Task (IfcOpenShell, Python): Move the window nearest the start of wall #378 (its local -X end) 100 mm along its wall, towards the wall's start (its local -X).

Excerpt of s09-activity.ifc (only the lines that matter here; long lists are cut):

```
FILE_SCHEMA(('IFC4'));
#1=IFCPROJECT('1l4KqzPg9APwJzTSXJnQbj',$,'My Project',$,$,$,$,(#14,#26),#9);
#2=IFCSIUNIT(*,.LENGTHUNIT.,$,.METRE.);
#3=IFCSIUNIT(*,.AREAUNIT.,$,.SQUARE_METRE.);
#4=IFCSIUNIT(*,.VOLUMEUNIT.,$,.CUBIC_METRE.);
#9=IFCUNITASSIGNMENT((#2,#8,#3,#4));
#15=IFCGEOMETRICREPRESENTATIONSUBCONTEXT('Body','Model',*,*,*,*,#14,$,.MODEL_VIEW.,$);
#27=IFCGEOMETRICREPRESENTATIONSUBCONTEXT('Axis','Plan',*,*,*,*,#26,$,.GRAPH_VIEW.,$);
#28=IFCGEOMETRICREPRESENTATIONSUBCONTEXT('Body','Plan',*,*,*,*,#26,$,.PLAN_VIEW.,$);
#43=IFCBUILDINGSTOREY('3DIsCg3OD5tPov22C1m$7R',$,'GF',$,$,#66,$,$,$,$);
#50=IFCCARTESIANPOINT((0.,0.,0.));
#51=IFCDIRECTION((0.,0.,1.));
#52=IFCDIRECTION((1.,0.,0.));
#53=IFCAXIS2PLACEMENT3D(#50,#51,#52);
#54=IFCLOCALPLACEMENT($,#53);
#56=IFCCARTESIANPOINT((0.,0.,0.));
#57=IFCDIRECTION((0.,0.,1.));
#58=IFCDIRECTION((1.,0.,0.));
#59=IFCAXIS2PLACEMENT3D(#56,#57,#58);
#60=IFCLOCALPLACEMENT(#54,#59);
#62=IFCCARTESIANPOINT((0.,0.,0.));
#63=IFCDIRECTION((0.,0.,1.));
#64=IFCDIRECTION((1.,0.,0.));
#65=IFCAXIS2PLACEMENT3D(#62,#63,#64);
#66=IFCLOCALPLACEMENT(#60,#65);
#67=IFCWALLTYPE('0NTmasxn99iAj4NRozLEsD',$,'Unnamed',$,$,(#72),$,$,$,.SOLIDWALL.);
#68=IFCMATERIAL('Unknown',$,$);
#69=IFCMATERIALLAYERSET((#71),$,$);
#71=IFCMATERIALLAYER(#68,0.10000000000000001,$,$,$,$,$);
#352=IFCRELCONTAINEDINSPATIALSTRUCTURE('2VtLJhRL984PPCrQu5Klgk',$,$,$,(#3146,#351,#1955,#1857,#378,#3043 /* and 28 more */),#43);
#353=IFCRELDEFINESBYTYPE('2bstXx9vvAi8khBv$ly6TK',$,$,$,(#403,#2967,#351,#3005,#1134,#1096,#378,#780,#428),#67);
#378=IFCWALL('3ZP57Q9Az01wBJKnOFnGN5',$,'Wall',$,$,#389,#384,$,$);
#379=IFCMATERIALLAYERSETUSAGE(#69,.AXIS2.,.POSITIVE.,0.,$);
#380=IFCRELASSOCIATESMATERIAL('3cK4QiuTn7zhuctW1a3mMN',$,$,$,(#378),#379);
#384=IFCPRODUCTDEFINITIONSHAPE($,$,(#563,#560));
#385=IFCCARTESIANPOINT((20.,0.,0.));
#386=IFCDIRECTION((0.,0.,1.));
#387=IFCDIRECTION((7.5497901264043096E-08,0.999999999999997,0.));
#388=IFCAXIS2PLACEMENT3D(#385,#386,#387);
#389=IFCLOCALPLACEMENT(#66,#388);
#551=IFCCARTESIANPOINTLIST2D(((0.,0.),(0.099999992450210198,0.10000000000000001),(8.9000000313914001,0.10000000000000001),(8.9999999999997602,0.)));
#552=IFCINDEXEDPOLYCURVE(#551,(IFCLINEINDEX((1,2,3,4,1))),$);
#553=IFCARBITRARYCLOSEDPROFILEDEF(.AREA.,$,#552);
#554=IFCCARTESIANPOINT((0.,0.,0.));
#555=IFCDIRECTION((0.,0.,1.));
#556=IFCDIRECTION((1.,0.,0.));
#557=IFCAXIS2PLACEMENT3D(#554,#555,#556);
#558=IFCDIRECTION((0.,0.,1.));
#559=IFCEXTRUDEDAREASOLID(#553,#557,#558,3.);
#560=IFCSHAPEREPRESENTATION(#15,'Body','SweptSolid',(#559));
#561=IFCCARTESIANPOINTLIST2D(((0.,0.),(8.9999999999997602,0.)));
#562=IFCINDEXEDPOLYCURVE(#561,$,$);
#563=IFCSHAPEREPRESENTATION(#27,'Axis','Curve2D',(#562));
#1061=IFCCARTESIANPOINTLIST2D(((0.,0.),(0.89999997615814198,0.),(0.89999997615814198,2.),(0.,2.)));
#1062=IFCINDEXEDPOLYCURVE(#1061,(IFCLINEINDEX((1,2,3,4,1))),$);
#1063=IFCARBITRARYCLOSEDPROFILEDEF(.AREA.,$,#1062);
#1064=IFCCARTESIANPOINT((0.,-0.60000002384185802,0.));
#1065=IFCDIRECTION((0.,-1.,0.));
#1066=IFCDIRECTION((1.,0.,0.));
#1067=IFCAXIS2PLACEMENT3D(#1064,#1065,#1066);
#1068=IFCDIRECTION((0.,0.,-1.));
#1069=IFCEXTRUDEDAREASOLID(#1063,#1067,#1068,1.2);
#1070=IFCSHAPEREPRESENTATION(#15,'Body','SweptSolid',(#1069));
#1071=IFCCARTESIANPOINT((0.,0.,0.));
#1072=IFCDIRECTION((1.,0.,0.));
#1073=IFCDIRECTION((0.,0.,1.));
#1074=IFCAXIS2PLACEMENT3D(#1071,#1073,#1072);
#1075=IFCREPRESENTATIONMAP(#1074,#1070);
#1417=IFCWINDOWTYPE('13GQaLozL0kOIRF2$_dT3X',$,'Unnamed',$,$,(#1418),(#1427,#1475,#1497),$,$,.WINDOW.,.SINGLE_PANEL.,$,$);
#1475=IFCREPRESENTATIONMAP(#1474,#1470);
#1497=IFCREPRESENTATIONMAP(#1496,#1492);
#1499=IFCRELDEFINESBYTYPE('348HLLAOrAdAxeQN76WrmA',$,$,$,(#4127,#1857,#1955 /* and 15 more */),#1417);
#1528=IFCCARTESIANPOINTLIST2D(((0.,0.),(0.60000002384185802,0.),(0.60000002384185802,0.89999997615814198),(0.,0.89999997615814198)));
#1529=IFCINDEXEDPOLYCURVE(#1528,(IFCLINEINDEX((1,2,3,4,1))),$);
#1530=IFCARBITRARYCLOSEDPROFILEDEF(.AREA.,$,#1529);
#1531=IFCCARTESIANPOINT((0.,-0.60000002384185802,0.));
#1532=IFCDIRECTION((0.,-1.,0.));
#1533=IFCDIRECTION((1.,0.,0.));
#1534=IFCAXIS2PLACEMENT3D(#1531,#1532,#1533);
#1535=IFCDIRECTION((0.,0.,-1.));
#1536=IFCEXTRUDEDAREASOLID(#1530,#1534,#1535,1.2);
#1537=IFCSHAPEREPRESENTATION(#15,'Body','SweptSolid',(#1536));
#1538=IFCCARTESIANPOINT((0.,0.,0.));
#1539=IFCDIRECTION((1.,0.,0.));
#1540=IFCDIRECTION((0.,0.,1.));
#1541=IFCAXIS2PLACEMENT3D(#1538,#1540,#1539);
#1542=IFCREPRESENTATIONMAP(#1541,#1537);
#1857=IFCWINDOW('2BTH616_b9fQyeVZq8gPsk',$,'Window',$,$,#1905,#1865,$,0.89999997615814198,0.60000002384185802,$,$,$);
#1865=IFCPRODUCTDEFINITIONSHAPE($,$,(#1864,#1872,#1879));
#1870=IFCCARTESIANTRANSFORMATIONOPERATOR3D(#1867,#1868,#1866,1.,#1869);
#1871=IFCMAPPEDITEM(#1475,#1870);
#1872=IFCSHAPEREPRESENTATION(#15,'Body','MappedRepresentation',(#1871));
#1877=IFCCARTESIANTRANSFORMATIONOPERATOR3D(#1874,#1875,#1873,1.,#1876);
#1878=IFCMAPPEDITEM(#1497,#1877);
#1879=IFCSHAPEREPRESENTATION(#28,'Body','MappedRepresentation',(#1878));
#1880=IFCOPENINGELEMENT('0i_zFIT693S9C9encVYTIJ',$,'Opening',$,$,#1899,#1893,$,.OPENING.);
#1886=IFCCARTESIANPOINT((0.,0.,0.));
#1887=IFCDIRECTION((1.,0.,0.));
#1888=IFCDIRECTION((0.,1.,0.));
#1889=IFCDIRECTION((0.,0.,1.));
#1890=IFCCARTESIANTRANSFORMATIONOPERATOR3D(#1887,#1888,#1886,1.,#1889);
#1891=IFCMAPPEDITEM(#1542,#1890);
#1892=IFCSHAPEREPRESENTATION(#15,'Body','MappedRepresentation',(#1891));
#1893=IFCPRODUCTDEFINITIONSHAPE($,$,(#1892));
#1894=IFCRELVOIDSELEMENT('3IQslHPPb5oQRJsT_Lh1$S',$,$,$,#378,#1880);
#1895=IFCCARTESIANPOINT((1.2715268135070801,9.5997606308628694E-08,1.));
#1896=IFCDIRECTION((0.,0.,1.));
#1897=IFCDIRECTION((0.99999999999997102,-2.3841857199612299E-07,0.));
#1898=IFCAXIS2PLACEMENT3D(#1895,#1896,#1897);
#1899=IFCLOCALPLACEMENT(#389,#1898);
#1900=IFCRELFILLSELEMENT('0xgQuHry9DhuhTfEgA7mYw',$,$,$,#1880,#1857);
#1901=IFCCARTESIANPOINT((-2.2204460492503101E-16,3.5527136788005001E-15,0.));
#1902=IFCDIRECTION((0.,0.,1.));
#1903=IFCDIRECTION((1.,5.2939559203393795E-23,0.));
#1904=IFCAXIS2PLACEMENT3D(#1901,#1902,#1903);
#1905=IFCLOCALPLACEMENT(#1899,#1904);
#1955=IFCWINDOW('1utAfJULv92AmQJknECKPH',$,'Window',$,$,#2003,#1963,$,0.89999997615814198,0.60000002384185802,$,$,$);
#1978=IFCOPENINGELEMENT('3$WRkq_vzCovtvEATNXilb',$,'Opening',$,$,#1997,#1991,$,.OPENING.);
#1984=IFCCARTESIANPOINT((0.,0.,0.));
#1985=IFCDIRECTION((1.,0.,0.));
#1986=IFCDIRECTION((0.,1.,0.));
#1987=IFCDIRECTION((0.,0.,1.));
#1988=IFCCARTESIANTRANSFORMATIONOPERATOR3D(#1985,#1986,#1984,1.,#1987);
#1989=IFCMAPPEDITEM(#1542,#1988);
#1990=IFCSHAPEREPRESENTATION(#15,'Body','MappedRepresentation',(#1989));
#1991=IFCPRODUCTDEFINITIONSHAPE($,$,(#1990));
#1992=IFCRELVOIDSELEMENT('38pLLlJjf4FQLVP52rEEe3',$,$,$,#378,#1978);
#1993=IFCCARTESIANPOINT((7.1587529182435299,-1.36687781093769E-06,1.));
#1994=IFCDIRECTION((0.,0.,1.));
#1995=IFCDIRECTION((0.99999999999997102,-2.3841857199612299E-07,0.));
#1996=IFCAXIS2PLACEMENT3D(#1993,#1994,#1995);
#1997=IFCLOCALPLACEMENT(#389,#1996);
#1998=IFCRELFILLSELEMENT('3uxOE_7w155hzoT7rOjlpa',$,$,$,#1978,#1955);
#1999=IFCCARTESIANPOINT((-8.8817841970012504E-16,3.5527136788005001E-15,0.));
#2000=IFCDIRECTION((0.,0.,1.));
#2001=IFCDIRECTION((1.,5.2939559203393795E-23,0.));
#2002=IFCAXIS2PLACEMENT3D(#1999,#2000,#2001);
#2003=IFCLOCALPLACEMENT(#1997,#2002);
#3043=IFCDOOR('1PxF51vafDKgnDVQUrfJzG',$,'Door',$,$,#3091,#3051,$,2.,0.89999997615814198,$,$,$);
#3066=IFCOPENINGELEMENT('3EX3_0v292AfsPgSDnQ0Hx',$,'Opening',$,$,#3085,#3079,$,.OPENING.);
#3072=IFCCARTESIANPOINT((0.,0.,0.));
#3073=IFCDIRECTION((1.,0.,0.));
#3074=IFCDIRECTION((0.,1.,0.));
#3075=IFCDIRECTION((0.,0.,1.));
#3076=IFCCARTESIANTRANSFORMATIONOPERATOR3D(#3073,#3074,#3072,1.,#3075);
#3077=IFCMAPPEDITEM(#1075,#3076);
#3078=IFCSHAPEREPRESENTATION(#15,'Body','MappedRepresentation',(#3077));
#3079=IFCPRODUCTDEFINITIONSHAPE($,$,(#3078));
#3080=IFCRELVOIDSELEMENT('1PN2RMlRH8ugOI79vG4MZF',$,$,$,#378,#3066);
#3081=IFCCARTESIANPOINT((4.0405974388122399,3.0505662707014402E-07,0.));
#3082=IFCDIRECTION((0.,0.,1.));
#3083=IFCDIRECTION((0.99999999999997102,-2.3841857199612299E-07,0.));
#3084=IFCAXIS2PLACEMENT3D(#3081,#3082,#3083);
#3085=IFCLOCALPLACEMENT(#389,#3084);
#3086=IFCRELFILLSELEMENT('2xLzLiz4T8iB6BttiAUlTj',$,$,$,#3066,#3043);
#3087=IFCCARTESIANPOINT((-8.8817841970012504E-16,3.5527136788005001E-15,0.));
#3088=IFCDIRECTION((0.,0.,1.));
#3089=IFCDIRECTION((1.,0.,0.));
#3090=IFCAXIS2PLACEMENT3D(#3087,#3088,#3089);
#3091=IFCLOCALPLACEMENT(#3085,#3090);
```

```python
import ifcopenshell
import ifcopenshell.api.geometry
import ifcopenshell.util.placement
import ifcopenshell.util.unit

model = ifcopenshell.open("s09-activity.ifc")
unit_scale = ifcopenshell.util.unit.calculate_unit_scale(model)

window = model.by_id(1857)
opening = window.FillsVoids[0].RelatingOpeningElement
wall = opening.VoidsElements[0].RelatingBuildingElement

wall_matrix = ifcopenshell.util.placement.get_local_placement(wall.ObjectPlacement)
shift = wall_matrix[:3, 0] * -0.1 / unit_scale
before = ifcopenshell.util.placement.get_local_placement(window.ObjectPlacement)[:3, 3].copy()

# The window is placed relative to its opening, so it follows when the opening moves.
matrix = ifcopenshell.util.placement.get_local_placement(opening.ObjectPlacement)
matrix[:3, 3] += shift
ifcopenshell.api.geometry.edit_object_placement(
    model, product=opening, matrix=matrix, is_si=False, should_transform_children=True
)

after = ifcopenshell.util.placement.get_local_placement(window.ObjectPlacement)[:3, 3]
print("window moved by", (after - before).round(3) + 0.0)

model.write("s09-activity_edited.ifc")
```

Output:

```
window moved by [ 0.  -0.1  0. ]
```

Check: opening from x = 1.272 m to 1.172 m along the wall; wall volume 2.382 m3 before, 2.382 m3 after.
